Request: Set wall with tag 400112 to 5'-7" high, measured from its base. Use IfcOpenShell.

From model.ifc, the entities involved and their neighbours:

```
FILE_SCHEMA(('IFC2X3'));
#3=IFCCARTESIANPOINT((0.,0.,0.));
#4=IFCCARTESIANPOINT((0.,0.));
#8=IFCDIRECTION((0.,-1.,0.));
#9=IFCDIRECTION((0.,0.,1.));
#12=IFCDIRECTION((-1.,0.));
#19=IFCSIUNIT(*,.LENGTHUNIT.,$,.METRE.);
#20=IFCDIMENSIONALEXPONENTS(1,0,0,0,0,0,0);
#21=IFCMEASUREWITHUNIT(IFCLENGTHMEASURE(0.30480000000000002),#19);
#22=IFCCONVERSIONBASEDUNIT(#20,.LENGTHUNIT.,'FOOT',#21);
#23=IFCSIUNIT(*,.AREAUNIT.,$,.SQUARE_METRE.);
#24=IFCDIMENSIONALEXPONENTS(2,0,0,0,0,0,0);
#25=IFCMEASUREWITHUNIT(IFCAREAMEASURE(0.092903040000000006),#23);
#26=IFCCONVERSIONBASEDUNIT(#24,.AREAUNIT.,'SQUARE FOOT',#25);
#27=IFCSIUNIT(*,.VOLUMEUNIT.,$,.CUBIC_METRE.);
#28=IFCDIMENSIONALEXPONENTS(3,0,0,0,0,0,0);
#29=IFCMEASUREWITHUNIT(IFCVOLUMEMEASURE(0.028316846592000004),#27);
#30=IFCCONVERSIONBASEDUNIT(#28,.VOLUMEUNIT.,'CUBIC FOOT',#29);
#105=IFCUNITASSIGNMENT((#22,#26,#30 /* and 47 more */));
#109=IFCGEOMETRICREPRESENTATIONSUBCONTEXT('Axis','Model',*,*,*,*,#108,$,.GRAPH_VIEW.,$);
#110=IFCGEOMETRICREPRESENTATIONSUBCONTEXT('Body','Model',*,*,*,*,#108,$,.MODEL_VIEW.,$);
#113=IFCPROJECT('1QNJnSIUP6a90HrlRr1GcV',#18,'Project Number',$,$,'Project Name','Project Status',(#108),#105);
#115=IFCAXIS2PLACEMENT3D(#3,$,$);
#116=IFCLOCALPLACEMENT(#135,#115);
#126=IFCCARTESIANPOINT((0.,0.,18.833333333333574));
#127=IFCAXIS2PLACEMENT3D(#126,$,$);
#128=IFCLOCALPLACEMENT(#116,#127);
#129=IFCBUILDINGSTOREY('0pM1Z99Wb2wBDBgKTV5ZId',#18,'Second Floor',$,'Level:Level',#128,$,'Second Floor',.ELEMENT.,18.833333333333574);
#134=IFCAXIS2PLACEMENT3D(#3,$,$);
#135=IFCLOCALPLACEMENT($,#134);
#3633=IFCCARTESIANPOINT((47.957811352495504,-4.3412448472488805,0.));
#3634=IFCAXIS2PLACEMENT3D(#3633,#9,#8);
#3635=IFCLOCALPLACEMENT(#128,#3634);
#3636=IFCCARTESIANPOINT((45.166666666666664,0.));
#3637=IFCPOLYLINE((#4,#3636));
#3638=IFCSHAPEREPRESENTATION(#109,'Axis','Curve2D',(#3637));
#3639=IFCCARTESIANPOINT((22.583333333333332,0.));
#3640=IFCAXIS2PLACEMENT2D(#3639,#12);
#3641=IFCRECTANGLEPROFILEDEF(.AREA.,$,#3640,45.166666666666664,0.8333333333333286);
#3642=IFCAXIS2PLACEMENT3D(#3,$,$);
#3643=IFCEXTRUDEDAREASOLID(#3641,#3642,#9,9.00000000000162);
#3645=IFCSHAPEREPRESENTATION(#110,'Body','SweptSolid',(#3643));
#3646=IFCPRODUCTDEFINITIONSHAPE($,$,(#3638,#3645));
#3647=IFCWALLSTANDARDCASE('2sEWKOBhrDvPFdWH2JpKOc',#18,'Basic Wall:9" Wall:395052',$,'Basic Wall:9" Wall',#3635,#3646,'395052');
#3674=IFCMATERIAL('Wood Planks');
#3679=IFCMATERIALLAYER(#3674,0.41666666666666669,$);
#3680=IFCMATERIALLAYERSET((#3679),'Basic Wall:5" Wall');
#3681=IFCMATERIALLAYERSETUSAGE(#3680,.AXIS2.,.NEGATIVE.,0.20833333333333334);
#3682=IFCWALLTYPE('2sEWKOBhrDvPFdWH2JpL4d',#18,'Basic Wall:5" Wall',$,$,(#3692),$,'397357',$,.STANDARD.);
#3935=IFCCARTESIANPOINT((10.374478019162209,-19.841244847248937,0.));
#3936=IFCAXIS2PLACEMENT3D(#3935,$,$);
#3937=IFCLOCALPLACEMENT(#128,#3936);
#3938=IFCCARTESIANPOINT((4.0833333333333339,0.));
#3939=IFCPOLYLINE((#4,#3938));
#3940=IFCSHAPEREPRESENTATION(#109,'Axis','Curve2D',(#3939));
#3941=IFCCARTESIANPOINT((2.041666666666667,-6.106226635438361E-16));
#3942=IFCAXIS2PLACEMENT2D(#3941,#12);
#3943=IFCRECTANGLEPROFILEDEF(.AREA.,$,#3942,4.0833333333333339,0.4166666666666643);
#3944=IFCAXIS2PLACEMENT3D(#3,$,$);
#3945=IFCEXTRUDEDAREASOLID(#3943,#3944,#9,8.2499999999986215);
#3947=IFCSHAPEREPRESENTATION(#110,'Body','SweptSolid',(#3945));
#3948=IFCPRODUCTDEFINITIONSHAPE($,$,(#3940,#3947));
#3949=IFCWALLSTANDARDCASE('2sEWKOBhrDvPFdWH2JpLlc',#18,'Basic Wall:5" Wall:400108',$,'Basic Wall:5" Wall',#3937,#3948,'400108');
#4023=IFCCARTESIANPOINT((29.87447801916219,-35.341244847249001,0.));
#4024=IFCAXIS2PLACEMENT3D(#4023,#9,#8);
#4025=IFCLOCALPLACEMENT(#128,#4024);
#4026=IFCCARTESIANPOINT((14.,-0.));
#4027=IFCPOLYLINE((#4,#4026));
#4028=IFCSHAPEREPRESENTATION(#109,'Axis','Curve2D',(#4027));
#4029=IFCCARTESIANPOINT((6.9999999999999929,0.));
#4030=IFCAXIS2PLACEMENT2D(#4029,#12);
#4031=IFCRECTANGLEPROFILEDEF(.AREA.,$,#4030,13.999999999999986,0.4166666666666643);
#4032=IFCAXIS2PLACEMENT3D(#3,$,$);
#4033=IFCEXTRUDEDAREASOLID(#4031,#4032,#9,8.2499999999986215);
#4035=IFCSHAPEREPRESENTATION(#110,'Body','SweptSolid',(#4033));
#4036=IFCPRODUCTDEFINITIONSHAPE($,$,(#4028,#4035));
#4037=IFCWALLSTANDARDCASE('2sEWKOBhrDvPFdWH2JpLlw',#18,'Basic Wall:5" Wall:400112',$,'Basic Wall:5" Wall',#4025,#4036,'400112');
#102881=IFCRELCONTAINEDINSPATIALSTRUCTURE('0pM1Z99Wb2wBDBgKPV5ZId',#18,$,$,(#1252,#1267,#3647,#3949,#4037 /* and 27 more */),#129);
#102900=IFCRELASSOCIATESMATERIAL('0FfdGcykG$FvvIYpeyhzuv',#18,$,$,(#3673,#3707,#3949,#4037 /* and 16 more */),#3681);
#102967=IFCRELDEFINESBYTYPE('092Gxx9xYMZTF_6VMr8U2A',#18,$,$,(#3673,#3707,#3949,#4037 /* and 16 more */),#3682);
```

```python
import ifcopenshell
import ifcopenshell.geom
import ifcopenshell.util.representation
import ifcopenshell.util.shape
import ifcopenshell.util.unit

model = ifcopenshell.open("model.ifc")
unit_scale = ifcopenshell.util.unit.calculate_unit_scale(model)
settings = ifcopenshell.geom.settings()


def volume(element):
    """Net volume in cubic metres, openings subtracted."""
    shape = ifcopenshell.geom.create_shape(settings, element)
    return ifcopenshell.util.shape.get_volume(shape.geometry)


wall = model.by_guid("2sEWKOBhrDvPFdWH2JpLlw")
before = volume(wall)

body = ifcopenshell.util.representation.get_representation(wall, "Model", "Body")
solid = body.Items[0]
old_height = solid.Depth
solid.Depth = 67 * 0.0254 / unit_scale
after = volume(wall)

print(f"height {old_height:g} -> {solid.Depth:g}, volume {before:.3f} -> {after:.3f} m3")

model.write("model_updated.ifc")
```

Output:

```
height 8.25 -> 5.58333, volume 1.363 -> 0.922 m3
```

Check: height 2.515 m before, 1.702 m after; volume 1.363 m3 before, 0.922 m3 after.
